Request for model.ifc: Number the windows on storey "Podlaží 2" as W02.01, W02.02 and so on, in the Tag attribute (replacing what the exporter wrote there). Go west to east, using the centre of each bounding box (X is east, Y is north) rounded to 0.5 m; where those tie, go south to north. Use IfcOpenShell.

First a look at what the model holds.

```python
import ifcopenshell
import ifcopenshell.util.element
import ifcopenshell.util.placement

model = ifcopenshell.open("model.ifc")
print(model.schema)
storey = next(s for s in model.by_type("IfcBuildingStorey") if s.Name == "Podlaží 2")
windows = [e for e in ifcopenshell.util.element.get_decomposition(storey) if e.is_a("IfcWindow")]
for e in sorted(windows, key=lambda e: e.id()):
    origin = ifcopenshell.util.placement.get_local_placement(e.ObjectPlacement)[:3, 3]
    print(e.id(), e.Tag, e.Name, origin.round(2) + 0.0, sep=" | ")
```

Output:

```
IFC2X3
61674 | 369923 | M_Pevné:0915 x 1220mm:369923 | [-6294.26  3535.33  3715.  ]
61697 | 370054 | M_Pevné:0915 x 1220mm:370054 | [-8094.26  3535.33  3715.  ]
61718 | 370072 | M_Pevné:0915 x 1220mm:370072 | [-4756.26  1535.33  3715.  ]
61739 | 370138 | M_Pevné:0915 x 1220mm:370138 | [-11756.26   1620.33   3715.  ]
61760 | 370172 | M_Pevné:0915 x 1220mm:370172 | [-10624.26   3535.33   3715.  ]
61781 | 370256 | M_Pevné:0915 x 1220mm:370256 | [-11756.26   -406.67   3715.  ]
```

```python
import ifcopenshell
import ifcopenshell.geom
import ifcopenshell.util.element
import ifcopenshell.util.shape

model = ifcopenshell.open("model.ifc")
settings = ifcopenshell.geom.settings()
settings.set("use-world-coords", True)


def centre(element):
    shape = ifcopenshell.geom.create_shape(settings, element)
    return ifcopenshell.util.shape.get_bbox_centroid(shape.geometry)


storey = next(s for s in model.by_type("IfcBuildingStorey") if s.Name == "Podlaží 2")
windows = [e for e in ifcopenshell.util.element.get_decomposition(storey) if e.is_a("IfcWindow")]

# Insertion points can sit at a corner or the storey origin, so sort by the geometry (in metres).
centres = {e: centre(e) for e in windows}
windows.sort(key=lambda e: (round(centres[e][0] / 0.5), centres[e][1]))

for i, e in enumerate(windows, start=1):
    number = f"W02.{i:02d}"
    e.Tag = number
    print(e.id(), number)

model.write("model_edited.ifc")
```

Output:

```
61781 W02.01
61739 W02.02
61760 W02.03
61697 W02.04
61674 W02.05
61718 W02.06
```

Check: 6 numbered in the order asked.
